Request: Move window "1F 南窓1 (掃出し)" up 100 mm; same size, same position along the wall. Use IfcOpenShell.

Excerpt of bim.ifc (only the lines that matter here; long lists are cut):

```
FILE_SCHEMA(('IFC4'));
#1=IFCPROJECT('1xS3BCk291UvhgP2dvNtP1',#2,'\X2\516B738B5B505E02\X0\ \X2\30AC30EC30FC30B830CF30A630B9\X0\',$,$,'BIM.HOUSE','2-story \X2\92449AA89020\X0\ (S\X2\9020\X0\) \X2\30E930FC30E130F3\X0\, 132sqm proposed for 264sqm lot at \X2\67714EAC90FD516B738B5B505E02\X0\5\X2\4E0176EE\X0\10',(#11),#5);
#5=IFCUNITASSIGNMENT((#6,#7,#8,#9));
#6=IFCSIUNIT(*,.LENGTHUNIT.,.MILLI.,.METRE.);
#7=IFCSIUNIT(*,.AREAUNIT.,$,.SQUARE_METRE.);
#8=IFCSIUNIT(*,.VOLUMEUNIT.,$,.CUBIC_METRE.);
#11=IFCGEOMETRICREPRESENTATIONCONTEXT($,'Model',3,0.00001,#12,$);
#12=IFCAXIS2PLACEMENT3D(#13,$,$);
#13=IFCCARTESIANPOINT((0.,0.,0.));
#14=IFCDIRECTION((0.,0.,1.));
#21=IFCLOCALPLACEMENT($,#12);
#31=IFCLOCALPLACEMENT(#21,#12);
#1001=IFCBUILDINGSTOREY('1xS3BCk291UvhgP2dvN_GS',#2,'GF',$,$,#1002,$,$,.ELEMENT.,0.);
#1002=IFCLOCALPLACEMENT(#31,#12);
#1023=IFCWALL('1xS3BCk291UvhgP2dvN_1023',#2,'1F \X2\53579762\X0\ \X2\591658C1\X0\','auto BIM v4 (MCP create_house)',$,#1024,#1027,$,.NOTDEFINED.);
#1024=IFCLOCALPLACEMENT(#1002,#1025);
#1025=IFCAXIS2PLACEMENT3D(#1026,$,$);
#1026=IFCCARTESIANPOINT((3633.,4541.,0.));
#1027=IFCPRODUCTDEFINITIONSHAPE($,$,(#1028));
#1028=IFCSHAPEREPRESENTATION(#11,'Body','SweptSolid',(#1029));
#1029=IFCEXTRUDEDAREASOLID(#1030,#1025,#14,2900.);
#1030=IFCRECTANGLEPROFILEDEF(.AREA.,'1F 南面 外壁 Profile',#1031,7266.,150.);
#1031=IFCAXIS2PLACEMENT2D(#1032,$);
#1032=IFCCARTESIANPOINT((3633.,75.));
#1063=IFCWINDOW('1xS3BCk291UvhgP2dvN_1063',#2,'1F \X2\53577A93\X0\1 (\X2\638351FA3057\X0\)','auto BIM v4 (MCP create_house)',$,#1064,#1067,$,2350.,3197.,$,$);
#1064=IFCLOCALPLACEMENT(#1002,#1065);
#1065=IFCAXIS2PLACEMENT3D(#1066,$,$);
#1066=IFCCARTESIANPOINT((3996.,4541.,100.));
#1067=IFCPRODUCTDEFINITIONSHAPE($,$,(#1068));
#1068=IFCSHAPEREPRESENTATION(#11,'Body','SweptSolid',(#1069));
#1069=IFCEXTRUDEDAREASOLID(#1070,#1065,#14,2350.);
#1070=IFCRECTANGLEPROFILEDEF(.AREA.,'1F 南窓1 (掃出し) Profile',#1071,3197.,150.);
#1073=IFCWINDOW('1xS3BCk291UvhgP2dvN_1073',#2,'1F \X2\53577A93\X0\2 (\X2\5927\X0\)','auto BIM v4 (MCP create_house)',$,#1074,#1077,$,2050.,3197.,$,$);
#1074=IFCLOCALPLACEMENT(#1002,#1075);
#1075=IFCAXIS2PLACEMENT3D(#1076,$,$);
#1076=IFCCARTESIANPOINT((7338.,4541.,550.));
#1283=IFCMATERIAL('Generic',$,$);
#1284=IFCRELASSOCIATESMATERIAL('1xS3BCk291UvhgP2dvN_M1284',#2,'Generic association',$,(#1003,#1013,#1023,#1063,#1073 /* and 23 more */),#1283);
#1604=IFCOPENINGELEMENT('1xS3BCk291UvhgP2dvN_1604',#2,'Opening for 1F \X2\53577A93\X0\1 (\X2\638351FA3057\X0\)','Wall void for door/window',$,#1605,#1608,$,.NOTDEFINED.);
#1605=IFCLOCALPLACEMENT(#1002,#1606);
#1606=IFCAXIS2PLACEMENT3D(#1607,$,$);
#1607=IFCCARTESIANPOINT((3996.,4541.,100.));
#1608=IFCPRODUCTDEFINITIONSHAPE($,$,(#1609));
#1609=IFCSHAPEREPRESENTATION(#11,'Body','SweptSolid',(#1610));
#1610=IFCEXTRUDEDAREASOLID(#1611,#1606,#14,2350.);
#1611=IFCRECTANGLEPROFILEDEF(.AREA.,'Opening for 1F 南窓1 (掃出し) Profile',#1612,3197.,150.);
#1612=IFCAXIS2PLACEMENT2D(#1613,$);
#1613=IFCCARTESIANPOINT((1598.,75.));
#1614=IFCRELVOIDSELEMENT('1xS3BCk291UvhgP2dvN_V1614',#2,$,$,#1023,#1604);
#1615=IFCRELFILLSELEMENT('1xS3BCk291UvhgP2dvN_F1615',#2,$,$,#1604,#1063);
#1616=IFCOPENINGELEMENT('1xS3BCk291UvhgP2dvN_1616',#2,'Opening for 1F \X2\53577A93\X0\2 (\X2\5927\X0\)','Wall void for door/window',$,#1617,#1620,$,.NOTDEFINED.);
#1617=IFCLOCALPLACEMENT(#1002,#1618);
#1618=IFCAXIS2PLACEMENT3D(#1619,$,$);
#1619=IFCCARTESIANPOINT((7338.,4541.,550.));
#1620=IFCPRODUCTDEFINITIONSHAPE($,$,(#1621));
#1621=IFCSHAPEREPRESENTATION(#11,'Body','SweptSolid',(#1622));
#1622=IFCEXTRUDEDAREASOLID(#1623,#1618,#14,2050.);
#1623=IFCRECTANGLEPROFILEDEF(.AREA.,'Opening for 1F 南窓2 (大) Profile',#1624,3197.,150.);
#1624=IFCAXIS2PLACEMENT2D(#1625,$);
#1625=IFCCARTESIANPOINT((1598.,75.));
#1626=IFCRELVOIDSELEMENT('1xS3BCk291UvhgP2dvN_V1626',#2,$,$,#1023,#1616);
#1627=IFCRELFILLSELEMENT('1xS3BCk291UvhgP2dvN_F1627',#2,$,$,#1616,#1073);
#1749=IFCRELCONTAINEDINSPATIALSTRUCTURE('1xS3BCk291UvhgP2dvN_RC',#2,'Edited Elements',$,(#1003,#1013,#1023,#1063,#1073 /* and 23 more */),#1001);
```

```python
import numpy as np
import ifcopenshell
import ifcopenshell.api.geometry
import ifcopenshell.util.placement
import ifcopenshell.util.unit

model = ifcopenshell.open("bim.ifc")
unit_scale = ifcopenshell.util.unit.calculate_unit_scale(model)

window = model.by_guid("1xS3BCk291UvhgP2dvN_1063")
opening = window.FillsVoids[0].RelatingOpeningElement
dz = 100.0

shift = np.array([0.0, 0.0, dz])
# The window is not placed relative to its opening, so move both.
for product in (opening, window):
    matrix = ifcopenshell.util.placement.get_local_placement(product.ObjectPlacement)
    matrix[:3, 3] += shift
    ifcopenshell.api.geometry.edit_object_placement(model, product=product, matrix=matrix, is_si=False)

print(f"moved by {dz * unit_scale:+.3f} m")

model.write("bim_edited.ifc")
```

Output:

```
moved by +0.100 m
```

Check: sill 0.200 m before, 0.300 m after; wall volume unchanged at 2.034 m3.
